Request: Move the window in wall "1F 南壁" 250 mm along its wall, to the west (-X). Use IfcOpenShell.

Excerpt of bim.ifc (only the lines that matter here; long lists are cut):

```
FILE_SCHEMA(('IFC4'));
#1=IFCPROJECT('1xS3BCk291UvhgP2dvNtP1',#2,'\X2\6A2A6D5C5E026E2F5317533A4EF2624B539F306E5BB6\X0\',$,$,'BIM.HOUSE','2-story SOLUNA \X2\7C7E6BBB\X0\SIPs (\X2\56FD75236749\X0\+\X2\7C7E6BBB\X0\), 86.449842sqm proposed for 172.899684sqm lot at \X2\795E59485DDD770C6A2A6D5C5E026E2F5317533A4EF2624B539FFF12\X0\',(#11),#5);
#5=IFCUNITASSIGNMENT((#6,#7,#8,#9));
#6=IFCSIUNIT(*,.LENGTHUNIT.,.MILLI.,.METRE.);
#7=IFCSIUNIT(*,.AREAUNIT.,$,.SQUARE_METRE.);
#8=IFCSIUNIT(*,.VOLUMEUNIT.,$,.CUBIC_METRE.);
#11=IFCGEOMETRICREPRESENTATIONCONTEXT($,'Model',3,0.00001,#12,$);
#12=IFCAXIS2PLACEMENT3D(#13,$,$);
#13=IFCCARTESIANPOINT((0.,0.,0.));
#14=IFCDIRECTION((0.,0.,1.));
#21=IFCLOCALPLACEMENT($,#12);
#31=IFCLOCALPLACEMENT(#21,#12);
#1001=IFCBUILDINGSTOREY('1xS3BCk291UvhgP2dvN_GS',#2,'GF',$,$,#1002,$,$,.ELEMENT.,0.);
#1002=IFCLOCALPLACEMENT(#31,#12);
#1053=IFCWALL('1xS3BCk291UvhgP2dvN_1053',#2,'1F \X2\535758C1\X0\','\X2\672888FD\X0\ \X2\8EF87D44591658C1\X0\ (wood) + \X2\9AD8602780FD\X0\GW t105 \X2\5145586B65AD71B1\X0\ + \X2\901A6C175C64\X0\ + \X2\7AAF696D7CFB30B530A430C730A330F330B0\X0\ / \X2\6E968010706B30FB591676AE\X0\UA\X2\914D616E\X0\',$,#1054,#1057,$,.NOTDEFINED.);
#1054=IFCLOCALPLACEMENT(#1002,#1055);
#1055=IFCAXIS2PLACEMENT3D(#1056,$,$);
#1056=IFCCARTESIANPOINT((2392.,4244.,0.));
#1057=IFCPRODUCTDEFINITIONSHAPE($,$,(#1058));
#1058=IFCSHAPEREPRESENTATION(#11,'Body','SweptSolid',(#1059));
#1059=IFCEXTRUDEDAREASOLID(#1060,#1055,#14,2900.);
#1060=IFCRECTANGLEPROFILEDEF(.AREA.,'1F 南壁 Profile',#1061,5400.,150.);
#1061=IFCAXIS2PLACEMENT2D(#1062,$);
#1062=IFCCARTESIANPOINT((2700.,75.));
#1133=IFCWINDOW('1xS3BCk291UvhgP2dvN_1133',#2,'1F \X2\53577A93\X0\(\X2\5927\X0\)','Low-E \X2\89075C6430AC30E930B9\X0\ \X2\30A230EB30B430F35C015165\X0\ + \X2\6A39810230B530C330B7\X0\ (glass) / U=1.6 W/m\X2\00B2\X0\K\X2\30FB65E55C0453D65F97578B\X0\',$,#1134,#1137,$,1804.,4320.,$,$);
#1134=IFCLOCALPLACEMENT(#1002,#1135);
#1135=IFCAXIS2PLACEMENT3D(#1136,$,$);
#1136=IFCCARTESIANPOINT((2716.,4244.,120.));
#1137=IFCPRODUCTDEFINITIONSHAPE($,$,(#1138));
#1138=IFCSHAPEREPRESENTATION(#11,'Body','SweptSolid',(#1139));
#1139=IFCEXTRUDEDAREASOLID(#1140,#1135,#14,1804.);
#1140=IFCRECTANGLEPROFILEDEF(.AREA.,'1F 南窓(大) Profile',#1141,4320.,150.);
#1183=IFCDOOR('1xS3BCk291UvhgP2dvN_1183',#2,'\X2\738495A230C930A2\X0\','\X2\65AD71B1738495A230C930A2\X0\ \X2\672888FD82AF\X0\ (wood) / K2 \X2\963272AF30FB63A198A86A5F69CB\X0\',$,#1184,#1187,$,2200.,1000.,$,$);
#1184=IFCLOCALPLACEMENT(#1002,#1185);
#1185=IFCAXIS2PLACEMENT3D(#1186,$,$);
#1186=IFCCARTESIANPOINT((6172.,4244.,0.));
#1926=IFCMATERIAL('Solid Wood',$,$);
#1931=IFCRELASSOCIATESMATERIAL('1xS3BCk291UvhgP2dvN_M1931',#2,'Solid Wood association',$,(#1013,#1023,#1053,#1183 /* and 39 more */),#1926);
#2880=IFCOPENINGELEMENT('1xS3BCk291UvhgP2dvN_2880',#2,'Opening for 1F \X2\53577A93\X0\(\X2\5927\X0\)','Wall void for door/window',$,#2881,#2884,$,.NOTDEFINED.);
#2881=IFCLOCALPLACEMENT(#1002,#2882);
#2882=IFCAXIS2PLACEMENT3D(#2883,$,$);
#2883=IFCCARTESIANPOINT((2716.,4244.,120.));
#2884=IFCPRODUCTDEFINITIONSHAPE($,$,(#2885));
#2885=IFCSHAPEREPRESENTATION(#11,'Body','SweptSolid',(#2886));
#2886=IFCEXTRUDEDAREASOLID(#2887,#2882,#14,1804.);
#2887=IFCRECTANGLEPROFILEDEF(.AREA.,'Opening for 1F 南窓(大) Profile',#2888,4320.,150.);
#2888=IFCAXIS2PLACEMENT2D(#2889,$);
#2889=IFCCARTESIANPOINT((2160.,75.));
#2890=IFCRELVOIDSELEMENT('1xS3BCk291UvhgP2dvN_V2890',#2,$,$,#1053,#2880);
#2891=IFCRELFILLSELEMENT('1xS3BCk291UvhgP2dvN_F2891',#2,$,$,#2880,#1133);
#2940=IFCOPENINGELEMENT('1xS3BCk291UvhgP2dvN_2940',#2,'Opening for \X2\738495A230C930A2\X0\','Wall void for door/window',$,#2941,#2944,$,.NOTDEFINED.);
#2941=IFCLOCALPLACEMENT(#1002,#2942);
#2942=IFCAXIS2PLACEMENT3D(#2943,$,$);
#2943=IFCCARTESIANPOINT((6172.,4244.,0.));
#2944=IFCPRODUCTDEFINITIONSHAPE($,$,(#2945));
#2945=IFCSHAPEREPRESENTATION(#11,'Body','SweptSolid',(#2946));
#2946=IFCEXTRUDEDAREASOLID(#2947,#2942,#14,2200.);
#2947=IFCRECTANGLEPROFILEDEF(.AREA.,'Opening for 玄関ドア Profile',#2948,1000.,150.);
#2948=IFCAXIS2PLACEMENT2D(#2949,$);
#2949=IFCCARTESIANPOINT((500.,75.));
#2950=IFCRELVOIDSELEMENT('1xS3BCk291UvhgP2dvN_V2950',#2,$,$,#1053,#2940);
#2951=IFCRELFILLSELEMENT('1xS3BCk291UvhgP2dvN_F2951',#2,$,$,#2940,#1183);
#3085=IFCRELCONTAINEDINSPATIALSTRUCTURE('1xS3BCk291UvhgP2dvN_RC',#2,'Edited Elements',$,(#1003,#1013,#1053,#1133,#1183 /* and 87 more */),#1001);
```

```python
import ifcopenshell
import ifcopenshell.api.geometry
import ifcopenshell.util.placement

model = ifcopenshell.open("bim.ifc")

window = model.by_guid("1xS3BCk291UvhgP2dvN_1133")
opening = window.FillsVoids[0].RelatingOpeningElement
wall = opening.VoidsElements[0].RelatingBuildingElement

wall_matrix = ifcopenshell.util.placement.get_local_placement(wall.ObjectPlacement)
shift = wall_matrix[:3, 0] * -250.0
before = ifcopenshell.util.placement.get_local_placement(window.ObjectPlacement)[:3, 3].copy()

# The window is not placed relative to its opening, so move both.
for product in (opening, window):
    matrix = ifcopenshell.util.placement.get_local_placement(product.ObjectPlacement)
    matrix[:3, 3] += shift
    ifcopenshell.api.geometry.edit_object_placement(model, product=product, matrix=matrix, is_si=False)

after = ifcopenshell.util.placement.get_local_placement(window.ObjectPlacement)[:3, 3]
print("window moved by", (after - before).round(3) + 0.0)

model.write("bim_v2.ifc")
```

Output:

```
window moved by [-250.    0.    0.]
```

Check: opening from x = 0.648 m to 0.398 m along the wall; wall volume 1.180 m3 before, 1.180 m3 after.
